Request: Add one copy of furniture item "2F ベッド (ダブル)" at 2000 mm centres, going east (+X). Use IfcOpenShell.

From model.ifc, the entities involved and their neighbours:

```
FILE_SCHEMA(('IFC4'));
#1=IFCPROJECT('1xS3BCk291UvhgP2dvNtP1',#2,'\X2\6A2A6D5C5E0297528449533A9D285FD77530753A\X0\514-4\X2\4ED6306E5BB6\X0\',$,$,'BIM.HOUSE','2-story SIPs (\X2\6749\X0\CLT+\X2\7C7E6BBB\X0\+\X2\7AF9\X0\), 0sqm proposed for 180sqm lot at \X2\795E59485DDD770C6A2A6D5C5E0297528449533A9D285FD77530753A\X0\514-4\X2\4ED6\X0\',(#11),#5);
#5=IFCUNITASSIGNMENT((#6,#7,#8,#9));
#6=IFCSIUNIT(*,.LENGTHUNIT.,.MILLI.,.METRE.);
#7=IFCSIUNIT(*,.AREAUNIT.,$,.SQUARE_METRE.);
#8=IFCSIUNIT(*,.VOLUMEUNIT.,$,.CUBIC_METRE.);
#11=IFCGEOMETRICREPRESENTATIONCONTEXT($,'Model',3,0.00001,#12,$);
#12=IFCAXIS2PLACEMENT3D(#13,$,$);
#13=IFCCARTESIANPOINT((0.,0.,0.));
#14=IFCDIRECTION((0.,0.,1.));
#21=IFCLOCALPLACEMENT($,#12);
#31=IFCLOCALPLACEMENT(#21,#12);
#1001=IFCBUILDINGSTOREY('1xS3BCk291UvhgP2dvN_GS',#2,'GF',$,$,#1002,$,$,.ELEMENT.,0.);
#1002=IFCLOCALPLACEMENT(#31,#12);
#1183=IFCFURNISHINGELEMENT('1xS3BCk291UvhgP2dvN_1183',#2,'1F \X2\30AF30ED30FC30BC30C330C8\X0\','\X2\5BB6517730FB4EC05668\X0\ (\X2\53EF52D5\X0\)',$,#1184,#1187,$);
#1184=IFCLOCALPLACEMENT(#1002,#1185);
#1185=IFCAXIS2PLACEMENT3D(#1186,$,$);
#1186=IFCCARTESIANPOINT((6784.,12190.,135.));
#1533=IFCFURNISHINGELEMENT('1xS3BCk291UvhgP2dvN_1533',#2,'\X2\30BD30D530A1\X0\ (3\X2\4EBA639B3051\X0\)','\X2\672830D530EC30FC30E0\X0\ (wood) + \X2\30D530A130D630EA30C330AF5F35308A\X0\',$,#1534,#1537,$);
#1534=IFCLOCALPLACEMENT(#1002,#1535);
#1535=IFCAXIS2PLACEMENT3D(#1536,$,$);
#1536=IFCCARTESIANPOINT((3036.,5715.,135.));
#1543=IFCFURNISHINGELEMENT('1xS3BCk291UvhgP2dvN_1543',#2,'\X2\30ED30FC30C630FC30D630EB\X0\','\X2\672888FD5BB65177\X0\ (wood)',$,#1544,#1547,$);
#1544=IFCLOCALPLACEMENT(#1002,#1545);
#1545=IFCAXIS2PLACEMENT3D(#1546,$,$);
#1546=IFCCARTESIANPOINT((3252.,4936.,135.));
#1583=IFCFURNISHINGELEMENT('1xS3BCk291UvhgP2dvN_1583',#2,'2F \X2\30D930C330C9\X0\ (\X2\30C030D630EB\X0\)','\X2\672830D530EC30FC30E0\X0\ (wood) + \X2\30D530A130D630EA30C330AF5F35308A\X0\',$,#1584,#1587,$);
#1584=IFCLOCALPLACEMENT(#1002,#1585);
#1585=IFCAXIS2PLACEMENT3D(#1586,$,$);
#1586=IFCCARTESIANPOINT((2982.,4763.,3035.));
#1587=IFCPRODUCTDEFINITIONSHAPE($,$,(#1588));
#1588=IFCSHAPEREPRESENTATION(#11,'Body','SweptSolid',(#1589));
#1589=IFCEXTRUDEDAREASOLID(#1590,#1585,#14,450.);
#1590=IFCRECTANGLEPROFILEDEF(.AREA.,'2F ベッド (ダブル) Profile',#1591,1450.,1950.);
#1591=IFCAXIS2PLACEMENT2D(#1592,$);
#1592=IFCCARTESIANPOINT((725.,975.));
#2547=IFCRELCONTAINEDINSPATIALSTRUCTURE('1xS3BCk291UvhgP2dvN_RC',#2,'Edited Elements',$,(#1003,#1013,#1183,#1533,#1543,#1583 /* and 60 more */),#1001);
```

```python
import numpy as np
import ifcopenshell
import ifcopenshell.api.geometry
import ifcopenshell.api.root
import ifcopenshell.util.element
import ifcopenshell.util.placement

model = ifcopenshell.open("model.ifc")


def reuse_history(source, copy):
    """copy_class also copies each property set's owner history, people and application; keep the originals."""
    for rel in copy.IsDefinedBy:
        if rel.is_a("IfcRelDefinesByProperties") and (history := rel.RelatingPropertyDefinition.OwnerHistory):
            rel.RelatingPropertyDefinition.OwnerHistory = source.OwnerHistory
            ifcopenshell.util.element.remove_deep2(model, history)


source = model.by_guid("1xS3BCk291UvhgP2dvN_1583")
base = ifcopenshell.util.placement.get_local_placement(source.ObjectPlacement)
step = np.array([1.0, 0.0, 0.0]) * 2000.0

for i in range(1, 2):
    copy = ifcopenshell.api.root.copy_class(model, product=source)
    copy.Representation = ifcopenshell.util.element.copy_deep(
        model, source.Representation, exclude=["IfcGeometricRepresentationContext", "IfcRepresentationMap"]
    )
    reuse_history(source, copy)
    matrix = base.copy()
    matrix[:3, 3] += i * step
    print("added at", matrix[:3, 3].round(3) + 0.0)
    ifcopenshell.api.geometry.edit_object_placement(model, product=copy, matrix=matrix, is_si=False)

model.write("model-out.ifc")
```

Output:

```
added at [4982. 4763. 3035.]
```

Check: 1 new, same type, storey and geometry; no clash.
